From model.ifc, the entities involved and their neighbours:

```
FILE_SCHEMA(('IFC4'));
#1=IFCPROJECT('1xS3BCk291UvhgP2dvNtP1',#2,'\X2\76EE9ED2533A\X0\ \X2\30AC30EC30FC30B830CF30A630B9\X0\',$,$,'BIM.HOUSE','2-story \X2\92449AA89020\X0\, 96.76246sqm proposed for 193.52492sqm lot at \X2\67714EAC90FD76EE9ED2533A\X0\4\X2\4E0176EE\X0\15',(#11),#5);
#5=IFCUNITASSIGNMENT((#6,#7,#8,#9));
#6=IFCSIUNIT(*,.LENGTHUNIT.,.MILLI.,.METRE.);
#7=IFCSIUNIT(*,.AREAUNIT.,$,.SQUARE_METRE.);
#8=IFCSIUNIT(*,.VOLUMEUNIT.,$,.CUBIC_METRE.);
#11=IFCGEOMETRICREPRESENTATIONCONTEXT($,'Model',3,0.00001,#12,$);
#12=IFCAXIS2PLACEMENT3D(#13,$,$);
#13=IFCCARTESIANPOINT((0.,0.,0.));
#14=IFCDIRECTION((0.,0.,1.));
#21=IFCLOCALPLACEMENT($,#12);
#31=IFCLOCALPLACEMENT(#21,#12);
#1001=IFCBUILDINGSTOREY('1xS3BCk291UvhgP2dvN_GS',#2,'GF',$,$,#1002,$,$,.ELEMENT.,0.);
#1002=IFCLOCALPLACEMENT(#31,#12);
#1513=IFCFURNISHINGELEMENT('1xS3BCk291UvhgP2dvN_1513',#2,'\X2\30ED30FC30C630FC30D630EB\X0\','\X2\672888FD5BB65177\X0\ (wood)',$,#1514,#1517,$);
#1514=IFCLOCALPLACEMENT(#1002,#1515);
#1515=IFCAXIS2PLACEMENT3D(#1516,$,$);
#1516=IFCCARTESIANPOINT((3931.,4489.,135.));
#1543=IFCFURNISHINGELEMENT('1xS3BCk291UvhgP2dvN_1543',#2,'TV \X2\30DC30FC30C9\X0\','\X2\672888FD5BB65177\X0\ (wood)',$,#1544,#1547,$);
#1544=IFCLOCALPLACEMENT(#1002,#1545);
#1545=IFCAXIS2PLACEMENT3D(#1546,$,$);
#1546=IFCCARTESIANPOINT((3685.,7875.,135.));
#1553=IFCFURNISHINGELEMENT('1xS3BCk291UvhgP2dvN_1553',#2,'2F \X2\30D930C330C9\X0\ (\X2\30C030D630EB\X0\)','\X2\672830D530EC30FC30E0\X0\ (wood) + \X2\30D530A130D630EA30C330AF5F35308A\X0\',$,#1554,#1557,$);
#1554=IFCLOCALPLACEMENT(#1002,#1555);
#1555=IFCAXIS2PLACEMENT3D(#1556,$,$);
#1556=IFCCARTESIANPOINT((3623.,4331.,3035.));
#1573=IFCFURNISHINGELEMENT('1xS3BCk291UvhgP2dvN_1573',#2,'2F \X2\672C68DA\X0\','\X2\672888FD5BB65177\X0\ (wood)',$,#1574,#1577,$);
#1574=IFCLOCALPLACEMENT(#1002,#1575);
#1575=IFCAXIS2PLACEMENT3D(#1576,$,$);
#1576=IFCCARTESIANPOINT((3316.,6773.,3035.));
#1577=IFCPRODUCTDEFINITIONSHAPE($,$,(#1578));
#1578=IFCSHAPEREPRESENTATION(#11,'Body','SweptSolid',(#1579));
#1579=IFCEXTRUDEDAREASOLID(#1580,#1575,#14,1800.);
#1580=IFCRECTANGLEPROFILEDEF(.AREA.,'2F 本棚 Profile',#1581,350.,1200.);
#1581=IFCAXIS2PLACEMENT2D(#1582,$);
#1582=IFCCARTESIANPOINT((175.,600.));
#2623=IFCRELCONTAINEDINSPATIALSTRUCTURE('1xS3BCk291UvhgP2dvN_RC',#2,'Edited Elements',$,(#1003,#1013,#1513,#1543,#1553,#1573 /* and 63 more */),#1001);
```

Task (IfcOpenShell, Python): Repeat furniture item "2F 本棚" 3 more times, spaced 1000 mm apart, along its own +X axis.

```python
import ifcopenshell
import ifcopenshell.api.geometry
import ifcopenshell.api.root
import ifcopenshell.util.element
import ifcopenshell.util.placement

model = ifcopenshell.open("model.ifc")


def reuse_history(source, copy):
    """copy_class also copies each property set's owner history, people and application; keep the originals."""
    for rel in copy.IsDefinedBy:
        if rel.is_a("IfcRelDefinesByProperties") and (history := rel.RelatingPropertyDefinition.OwnerHistory):
            rel.RelatingPropertyDefinition.OwnerHistory = source.OwnerHistory
            ifcopenshell.util.element.remove_deep2(model, history)


source = model.by_guid("1xS3BCk291UvhgP2dvN_1573")
base = ifcopenshell.util.placement.get_local_placement(source.ObjectPlacement)
step = base[:3, 0] * 1000.0

for i in range(1, 4):
    copy = ifcopenshell.api.root.copy_class(model, product=source)
    copy.Representation = ifcopenshell.util.element.copy_deep(
        model, source.Representation, exclude=["IfcGeometricRepresentationContext", "IfcRepresentationMap"]
    )
    reuse_history(source, copy)
    matrix = base.copy()
    matrix[:3, 3] += i * step
    print("added at", matrix[:3, 3].round(3) + 0.0)
    ifcopenshell.api.geometry.edit_object_placement(model, product=copy, matrix=matrix, is_si=False)

model.write("model_v2.ifc")
```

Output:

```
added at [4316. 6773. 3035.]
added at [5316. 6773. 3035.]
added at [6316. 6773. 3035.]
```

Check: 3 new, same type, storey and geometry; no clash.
